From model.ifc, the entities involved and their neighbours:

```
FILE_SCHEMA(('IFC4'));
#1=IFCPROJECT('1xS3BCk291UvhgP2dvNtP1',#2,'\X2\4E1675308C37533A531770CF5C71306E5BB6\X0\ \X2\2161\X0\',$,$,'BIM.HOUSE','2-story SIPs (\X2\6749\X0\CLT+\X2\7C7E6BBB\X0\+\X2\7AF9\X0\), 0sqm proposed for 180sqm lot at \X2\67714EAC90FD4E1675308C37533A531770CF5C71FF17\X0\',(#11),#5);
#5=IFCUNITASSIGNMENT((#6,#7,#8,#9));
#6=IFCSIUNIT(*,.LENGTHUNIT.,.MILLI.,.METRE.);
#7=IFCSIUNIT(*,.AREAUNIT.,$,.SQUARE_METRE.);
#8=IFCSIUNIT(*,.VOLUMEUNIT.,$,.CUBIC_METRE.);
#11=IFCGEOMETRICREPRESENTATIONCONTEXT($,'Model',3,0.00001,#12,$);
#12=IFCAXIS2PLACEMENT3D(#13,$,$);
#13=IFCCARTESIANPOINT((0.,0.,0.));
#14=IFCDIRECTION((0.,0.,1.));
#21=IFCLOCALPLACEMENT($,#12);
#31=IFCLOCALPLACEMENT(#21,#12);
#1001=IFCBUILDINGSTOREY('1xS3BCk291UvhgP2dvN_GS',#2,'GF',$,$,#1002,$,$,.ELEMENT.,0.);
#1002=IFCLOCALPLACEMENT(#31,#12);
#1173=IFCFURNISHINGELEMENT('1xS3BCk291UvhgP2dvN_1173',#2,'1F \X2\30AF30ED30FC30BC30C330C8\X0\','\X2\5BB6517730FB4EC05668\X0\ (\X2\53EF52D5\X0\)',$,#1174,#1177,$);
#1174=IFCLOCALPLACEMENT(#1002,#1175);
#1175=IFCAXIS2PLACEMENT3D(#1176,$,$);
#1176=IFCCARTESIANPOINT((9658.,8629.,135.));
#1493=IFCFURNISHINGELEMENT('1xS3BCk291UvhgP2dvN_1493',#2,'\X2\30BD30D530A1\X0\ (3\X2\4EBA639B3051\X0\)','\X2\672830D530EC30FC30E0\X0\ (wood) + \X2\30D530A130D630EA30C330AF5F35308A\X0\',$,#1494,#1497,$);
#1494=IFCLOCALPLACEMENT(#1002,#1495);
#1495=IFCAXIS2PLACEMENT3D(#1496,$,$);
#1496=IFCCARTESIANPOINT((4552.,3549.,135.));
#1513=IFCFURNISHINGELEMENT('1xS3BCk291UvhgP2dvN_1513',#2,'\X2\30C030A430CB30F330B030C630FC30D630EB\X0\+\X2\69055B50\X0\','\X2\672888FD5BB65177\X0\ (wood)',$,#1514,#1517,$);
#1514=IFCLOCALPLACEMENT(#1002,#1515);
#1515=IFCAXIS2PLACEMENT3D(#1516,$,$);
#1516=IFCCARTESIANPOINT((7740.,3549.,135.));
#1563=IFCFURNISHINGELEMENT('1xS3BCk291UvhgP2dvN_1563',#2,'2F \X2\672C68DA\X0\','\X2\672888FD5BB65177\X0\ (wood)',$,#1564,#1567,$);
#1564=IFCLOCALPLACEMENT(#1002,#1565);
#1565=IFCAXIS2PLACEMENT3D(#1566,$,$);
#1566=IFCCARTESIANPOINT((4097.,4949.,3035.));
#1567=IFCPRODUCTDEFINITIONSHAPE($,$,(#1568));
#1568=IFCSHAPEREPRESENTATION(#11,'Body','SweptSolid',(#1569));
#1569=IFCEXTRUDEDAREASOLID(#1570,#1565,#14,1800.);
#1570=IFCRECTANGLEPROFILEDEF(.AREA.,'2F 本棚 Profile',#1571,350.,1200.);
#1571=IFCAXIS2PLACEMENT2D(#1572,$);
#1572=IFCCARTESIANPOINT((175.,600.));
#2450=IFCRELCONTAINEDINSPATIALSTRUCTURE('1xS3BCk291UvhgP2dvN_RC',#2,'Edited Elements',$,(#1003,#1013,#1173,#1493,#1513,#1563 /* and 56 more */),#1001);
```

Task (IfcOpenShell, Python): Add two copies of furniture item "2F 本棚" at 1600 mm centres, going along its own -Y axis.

```python
import ifcopenshell
import ifcopenshell.api.geometry
import ifcopenshell.api.root
import ifcopenshell.util.element
import ifcopenshell.util.placement
import ifcopenshell.util.unit

model = ifcopenshell.open("model.ifc")
unit_scale = ifcopenshell.util.unit.calculate_unit_scale(model)


def reuse_history(source, copy):
    """copy_class also copies each property set's owner history, people and application; keep the originals."""
    for rel in copy.IsDefinedBy:
        if rel.is_a("IfcRelDefinesByProperties") and (history := rel.RelatingPropertyDefinition.OwnerHistory):
            rel.RelatingPropertyDefinition.OwnerHistory = source.OwnerHistory
            ifcopenshell.util.element.remove_deep2(model, history)


source = model.by_guid("1xS3BCk291UvhgP2dvN_1563")
base = ifcopenshell.util.placement.get_local_placement(source.ObjectPlacement)
step = -base[:3, 1] * 1.6 / unit_scale

for i in range(1, 3):
    copy = ifcopenshell.api.root.copy_class(model, product=source)
    copy.Representation = ifcopenshell.util.element.copy_deep(
        model, source.Representation, exclude=["IfcGeometricRepresentationContext", "IfcRepresentationMap"]
    )
    reuse_history(source, copy)
    matrix = base.copy()
    matrix[:3, 3] += i * step
    print("added at", matrix[:3, 3].round(3) + 0.0)
    ifcopenshell.api.geometry.edit_object_placement(model, product=copy, matrix=matrix, is_si=False)

model.write("model_v2.ifc")
```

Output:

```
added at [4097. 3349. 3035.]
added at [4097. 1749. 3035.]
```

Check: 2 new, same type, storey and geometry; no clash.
